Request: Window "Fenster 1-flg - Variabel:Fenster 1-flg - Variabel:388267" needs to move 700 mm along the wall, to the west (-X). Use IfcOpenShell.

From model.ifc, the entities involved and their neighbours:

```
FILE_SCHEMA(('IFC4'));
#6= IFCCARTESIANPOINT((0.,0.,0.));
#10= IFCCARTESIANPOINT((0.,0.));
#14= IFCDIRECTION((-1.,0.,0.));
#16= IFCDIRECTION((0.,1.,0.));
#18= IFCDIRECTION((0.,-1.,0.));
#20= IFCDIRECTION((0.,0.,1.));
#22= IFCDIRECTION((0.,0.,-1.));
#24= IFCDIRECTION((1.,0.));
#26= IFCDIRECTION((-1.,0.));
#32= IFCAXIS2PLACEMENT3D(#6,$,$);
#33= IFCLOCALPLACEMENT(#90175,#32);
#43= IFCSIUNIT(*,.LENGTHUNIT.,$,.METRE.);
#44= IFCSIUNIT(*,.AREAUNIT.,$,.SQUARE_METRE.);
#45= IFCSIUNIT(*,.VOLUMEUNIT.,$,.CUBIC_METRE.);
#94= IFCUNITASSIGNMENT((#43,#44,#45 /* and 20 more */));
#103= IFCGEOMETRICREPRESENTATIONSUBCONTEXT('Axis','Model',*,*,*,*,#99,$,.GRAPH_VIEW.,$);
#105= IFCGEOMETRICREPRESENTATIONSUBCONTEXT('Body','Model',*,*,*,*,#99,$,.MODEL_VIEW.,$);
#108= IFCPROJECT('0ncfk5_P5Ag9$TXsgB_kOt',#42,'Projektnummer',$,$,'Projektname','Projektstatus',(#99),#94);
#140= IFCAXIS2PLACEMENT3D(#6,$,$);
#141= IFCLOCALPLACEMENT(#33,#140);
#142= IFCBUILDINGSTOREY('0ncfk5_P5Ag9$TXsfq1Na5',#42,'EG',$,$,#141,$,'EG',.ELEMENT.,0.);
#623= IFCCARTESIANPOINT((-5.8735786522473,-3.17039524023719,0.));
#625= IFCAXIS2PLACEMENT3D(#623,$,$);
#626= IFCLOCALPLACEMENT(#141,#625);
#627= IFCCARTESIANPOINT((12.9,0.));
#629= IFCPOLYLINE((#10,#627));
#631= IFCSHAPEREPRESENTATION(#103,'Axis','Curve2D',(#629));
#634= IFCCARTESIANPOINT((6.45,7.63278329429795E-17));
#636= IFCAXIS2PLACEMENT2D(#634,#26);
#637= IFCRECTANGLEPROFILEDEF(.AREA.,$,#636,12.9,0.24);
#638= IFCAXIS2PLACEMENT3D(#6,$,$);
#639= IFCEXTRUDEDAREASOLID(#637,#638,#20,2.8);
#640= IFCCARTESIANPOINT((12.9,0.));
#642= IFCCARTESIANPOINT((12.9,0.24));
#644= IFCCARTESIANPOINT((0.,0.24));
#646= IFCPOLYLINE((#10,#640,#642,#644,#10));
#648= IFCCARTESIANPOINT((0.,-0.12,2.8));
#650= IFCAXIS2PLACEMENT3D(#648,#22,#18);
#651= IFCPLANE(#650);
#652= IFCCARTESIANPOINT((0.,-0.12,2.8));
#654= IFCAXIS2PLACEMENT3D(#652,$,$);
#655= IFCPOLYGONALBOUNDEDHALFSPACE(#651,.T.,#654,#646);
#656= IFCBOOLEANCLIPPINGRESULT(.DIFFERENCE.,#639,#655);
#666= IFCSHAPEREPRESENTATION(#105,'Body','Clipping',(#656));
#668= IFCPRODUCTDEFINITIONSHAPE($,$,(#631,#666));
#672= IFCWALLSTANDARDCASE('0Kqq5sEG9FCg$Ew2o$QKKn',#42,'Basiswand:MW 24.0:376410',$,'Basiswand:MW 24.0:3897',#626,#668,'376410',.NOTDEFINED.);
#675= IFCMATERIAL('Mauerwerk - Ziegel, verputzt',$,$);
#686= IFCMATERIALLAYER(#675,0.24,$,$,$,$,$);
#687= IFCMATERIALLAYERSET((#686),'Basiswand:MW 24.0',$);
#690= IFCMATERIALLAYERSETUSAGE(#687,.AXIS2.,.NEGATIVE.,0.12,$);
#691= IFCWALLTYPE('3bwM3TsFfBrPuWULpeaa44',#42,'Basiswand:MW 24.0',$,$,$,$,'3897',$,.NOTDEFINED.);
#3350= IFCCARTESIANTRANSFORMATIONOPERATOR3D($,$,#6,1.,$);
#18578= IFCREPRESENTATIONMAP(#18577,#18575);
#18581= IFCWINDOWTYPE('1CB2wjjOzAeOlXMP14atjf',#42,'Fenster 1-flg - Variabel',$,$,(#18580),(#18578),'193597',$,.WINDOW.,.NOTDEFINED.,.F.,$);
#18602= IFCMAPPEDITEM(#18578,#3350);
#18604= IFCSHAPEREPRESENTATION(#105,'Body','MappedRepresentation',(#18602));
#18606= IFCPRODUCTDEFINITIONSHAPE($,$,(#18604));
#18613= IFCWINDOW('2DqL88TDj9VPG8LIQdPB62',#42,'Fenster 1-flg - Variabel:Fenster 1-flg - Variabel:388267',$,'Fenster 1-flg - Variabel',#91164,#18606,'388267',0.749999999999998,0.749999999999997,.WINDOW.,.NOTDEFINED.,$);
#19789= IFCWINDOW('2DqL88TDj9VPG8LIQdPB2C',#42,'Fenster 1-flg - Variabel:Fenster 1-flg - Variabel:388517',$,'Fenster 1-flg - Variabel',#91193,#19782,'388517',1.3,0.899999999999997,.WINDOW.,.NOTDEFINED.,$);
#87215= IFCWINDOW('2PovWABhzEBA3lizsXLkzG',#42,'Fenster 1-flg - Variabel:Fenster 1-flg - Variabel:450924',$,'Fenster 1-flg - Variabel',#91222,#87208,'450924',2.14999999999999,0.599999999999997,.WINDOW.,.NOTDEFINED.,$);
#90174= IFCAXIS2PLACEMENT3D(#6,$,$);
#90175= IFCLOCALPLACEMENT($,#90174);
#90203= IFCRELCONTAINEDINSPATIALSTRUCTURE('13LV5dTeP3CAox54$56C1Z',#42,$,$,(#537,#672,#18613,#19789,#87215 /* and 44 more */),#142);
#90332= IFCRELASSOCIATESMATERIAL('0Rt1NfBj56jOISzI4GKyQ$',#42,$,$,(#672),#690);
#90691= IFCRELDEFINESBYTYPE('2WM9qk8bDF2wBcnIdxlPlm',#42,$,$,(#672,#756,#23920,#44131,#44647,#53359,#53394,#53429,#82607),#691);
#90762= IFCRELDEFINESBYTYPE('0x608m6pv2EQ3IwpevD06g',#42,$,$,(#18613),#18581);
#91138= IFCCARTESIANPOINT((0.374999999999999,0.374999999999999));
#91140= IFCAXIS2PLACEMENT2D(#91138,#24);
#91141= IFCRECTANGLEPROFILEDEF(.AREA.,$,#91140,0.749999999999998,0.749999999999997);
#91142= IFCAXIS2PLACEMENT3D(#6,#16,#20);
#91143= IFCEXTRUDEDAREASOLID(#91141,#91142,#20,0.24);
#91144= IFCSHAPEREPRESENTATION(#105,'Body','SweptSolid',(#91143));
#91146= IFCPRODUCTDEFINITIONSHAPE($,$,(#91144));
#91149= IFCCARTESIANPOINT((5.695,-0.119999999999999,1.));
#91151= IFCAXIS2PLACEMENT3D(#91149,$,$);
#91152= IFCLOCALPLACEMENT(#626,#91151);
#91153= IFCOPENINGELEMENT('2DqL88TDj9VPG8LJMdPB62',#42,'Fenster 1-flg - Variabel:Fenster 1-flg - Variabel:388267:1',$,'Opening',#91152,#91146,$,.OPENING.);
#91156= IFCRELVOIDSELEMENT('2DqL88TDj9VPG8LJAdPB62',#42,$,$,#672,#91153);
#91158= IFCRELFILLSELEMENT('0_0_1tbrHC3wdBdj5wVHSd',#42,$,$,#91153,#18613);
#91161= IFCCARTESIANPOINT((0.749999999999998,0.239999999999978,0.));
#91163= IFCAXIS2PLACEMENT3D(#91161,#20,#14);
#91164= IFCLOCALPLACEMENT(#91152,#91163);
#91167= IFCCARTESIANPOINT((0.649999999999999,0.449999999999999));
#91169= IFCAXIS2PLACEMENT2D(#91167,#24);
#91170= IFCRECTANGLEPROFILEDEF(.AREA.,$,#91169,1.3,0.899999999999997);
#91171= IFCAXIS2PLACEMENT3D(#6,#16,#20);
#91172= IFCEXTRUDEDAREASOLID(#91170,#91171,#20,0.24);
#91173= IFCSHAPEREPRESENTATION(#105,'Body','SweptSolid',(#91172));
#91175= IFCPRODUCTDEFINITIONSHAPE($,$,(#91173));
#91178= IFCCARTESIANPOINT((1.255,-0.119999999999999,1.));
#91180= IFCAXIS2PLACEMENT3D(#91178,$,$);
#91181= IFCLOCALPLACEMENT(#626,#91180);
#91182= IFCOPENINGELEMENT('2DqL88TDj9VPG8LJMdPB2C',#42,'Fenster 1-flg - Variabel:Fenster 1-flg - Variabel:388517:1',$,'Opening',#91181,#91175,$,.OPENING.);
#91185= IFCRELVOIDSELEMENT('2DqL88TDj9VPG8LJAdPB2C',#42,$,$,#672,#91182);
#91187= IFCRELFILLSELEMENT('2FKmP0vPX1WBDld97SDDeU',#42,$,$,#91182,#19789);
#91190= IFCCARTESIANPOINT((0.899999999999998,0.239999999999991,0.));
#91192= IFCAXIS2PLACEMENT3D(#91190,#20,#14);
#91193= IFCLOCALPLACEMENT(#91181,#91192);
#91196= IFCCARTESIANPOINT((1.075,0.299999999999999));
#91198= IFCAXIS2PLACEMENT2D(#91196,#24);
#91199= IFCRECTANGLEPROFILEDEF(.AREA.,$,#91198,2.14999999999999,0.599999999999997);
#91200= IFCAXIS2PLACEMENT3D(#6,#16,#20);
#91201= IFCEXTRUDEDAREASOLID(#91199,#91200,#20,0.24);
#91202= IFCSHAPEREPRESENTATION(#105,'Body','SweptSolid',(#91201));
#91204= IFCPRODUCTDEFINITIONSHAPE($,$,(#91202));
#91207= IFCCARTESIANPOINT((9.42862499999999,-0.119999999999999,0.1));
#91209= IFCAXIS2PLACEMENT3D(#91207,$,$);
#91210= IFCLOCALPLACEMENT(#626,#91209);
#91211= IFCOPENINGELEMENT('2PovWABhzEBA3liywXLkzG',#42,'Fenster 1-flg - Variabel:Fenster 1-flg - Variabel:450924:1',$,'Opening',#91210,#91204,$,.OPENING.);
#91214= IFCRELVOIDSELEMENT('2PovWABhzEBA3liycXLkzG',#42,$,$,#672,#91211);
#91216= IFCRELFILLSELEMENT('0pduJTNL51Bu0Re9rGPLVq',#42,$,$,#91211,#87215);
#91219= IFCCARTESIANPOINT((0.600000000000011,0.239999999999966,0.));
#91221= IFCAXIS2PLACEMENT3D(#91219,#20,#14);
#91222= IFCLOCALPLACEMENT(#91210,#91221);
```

```python
import ifcopenshell
import ifcopenshell.api.geometry
import ifcopenshell.util.placement
import ifcopenshell.util.unit

model = ifcopenshell.open("model.ifc")
unit_scale = ifcopenshell.util.unit.calculate_unit_scale(model)

window = model.by_id(18613)
opening = window.FillsVoids[0].RelatingOpeningElement
wall = opening.VoidsElements[0].RelatingBuildingElement

wall_matrix = ifcopenshell.util.placement.get_local_placement(wall.ObjectPlacement)
shift = wall_matrix[:3, 0] * -0.7 / unit_scale
before = ifcopenshell.util.placement.get_local_placement(window.ObjectPlacement)[:3, 3].copy()

# The window is placed relative to its opening, so it follows when the opening moves.
matrix = ifcopenshell.util.placement.get_local_placement(opening.ObjectPlacement)
matrix[:3, 3] += shift
ifcopenshell.api.geometry.edit_object_placement(
    model, product=opening, matrix=matrix, is_si=False, should_transform_children=True
)

after = ifcopenshell.util.placement.get_local_placement(window.ObjectPlacement)[:3, 3]
print("window moved by", (after - before).round(3) + 0.0)

model.write("model-out.ifc")
```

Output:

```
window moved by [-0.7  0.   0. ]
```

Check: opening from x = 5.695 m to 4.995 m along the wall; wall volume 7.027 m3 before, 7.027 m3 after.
